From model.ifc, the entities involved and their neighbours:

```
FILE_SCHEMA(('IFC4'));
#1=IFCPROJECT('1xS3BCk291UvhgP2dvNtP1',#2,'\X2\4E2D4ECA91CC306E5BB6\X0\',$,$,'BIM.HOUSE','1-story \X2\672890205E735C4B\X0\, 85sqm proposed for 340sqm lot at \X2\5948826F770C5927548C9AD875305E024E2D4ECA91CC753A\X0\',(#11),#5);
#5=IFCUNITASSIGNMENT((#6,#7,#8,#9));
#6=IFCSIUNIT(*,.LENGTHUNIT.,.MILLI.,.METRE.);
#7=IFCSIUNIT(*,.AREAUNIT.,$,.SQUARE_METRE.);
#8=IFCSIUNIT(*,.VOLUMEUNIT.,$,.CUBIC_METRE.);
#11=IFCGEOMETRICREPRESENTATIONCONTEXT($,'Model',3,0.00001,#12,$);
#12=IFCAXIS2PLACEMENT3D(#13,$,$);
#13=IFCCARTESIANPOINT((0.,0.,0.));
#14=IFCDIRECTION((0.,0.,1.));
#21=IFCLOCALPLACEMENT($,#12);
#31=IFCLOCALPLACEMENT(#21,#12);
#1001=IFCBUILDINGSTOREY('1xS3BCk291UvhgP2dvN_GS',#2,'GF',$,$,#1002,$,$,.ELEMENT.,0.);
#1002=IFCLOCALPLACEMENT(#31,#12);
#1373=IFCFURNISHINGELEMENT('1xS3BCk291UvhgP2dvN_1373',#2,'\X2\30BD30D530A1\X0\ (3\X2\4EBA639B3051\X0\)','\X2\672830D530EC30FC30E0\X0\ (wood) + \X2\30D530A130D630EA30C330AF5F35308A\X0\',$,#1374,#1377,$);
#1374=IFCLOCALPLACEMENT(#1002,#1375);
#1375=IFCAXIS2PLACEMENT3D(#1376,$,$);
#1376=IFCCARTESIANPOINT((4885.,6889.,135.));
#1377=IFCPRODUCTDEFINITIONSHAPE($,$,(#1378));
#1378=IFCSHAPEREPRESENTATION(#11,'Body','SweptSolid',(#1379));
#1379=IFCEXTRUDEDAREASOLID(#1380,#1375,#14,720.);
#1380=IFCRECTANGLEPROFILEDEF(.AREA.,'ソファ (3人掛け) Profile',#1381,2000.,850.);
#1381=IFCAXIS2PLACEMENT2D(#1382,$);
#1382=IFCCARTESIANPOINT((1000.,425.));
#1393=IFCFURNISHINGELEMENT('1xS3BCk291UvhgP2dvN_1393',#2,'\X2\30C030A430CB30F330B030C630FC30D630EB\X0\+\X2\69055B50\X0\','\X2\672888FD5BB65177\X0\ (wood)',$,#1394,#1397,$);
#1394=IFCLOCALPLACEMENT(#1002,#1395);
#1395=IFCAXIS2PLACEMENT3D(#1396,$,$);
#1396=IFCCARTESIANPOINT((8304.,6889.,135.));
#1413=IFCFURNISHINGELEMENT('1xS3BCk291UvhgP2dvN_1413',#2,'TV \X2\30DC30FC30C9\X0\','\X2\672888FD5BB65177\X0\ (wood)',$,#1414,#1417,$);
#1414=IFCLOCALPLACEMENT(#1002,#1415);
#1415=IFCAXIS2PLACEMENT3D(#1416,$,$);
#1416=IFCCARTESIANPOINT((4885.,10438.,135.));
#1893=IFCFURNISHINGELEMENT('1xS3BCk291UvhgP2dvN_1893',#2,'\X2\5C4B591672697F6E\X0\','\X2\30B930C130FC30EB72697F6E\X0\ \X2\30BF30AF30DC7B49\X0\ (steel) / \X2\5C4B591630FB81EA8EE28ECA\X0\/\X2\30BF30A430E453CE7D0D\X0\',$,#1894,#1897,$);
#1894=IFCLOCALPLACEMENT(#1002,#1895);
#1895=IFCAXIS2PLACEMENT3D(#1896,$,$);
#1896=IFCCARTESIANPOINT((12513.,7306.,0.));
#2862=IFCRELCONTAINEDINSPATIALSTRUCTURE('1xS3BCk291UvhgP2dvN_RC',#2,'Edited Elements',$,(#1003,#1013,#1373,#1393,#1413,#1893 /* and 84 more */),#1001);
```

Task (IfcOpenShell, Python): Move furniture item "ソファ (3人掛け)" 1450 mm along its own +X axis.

```python
import ifcopenshell
import ifcopenshell.api.geometry
import ifcopenshell.util.placement
import ifcopenshell.util.unit

model = ifcopenshell.open("model.ifc")
unit_scale = ifcopenshell.util.unit.calculate_unit_scale(model)

item = model.by_guid("1xS3BCk291UvhgP2dvN_1373")
matrix = ifcopenshell.util.placement.get_local_placement(item.ObjectPlacement)
matrix[:3, 3] += matrix[:3, 0] * 1.45 / unit_scale
ifcopenshell.api.geometry.edit_object_placement(model, product=item, matrix=matrix, is_si=False)

print(ifcopenshell.util.placement.get_local_placement(item.ObjectPlacement).round(3) + 0.0)

model.write("model_updated.ifc")
```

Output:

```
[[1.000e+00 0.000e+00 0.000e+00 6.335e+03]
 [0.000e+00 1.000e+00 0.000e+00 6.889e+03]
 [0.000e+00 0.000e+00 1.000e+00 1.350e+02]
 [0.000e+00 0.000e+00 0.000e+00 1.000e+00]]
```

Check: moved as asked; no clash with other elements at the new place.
